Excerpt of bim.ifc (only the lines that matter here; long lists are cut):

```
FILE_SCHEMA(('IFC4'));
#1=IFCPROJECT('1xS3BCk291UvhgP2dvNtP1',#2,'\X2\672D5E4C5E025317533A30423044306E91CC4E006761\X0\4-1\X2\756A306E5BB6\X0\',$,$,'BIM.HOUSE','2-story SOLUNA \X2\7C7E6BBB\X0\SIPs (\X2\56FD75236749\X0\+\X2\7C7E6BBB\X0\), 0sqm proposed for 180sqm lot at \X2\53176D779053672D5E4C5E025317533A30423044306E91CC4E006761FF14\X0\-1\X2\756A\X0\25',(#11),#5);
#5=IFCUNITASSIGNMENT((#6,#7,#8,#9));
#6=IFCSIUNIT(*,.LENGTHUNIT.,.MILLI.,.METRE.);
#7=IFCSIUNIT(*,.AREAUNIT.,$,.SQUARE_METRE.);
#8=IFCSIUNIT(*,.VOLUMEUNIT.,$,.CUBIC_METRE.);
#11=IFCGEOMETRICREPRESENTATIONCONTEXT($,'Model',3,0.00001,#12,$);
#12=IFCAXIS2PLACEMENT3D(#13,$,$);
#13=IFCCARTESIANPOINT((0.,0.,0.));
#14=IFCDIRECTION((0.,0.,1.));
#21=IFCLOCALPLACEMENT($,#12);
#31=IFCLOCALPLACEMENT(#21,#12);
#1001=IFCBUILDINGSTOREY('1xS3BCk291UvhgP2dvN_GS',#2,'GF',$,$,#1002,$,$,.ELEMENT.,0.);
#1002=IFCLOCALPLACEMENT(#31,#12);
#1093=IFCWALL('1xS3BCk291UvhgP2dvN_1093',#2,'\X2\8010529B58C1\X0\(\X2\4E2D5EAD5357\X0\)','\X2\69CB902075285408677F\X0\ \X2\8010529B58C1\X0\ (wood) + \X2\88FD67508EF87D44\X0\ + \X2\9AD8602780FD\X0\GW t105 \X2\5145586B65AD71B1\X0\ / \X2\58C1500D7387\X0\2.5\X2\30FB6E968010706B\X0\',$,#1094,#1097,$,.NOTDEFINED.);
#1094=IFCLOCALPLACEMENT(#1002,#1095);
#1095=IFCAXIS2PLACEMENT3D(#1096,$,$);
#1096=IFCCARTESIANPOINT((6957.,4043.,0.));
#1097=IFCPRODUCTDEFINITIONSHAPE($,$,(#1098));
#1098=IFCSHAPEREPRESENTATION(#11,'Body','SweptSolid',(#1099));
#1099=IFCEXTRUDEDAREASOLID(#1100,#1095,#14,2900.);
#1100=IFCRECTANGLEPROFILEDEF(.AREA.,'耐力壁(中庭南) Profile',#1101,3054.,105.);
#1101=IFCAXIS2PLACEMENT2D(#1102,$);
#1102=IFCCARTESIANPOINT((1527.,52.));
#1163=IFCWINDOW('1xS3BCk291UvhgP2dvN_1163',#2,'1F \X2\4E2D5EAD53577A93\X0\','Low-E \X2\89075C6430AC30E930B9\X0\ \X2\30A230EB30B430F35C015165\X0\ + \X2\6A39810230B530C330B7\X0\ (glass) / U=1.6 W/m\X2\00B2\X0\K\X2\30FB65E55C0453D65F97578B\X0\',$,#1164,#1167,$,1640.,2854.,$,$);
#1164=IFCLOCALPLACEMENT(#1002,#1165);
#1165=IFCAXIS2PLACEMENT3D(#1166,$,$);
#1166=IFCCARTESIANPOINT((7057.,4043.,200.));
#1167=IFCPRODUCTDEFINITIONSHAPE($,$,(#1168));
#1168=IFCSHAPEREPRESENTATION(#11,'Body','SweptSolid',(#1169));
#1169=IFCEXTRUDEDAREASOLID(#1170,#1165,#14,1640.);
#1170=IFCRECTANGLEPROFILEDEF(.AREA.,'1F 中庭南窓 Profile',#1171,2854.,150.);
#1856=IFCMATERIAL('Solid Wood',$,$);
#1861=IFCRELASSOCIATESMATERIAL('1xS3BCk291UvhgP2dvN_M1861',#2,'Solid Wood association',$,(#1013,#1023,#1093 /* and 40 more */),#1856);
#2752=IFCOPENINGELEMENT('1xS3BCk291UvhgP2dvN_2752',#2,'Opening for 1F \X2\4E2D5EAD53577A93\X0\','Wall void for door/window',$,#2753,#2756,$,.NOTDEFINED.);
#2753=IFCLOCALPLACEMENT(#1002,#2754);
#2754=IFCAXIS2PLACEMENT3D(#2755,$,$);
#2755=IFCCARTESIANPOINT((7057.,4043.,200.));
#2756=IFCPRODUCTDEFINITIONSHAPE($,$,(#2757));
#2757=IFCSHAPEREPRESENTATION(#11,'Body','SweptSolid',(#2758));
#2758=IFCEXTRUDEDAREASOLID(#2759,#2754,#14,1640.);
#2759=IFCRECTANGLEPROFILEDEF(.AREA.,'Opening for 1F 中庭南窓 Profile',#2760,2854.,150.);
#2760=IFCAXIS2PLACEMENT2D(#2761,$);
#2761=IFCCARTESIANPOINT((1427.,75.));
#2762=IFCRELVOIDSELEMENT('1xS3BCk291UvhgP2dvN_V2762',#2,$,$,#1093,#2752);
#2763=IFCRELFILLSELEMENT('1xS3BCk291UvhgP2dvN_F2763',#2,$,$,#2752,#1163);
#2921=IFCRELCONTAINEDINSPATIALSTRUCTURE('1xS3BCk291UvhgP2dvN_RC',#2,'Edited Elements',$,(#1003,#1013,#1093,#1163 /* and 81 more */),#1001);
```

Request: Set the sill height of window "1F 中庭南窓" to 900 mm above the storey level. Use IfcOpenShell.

```python
import numpy as np
import ifcopenshell
import ifcopenshell.api.geometry
import ifcopenshell.geom
import ifcopenshell.util.element
import ifcopenshell.util.placement
import ifcopenshell.util.shape
import ifcopenshell.util.unit

model = ifcopenshell.open("bim.ifc")
unit_scale = ifcopenshell.util.unit.calculate_unit_scale(model)

window = model.by_guid("1xS3BCk291UvhgP2dvN_1163")
opening = window.FillsVoids[0].RelatingOpeningElement
storey = ifcopenshell.util.element.get_container(window, ifc_class="IfcBuildingStorey")
level = ifcopenshell.util.placement.get_local_placement(storey.ObjectPlacement)[2, 3]

# The opening's origin need not be at the sill, so measure its lowest point.
shape = ifcopenshell.geom.create_shape(ifcopenshell.geom.settings(), opening)
bottom = ifcopenshell.util.shape.get_shape_bottom_elevation(shape, shape.geometry) / unit_scale
dz = level + 0.9 / unit_scale - bottom

shift = np.array([0.0, 0.0, dz])
# The window is not placed relative to its opening, so move both.
for product in (opening, window):
    matrix = ifcopenshell.util.placement.get_local_placement(product.ObjectPlacement)
    matrix[:3, 3] += shift
    ifcopenshell.api.geometry.edit_object_placement(model, product=product, matrix=matrix, is_si=False)

print(f"moved by {dz * unit_scale:+.3f} m")

model.write("bim_rev.ifc")
```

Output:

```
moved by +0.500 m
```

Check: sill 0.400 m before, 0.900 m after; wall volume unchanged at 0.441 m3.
